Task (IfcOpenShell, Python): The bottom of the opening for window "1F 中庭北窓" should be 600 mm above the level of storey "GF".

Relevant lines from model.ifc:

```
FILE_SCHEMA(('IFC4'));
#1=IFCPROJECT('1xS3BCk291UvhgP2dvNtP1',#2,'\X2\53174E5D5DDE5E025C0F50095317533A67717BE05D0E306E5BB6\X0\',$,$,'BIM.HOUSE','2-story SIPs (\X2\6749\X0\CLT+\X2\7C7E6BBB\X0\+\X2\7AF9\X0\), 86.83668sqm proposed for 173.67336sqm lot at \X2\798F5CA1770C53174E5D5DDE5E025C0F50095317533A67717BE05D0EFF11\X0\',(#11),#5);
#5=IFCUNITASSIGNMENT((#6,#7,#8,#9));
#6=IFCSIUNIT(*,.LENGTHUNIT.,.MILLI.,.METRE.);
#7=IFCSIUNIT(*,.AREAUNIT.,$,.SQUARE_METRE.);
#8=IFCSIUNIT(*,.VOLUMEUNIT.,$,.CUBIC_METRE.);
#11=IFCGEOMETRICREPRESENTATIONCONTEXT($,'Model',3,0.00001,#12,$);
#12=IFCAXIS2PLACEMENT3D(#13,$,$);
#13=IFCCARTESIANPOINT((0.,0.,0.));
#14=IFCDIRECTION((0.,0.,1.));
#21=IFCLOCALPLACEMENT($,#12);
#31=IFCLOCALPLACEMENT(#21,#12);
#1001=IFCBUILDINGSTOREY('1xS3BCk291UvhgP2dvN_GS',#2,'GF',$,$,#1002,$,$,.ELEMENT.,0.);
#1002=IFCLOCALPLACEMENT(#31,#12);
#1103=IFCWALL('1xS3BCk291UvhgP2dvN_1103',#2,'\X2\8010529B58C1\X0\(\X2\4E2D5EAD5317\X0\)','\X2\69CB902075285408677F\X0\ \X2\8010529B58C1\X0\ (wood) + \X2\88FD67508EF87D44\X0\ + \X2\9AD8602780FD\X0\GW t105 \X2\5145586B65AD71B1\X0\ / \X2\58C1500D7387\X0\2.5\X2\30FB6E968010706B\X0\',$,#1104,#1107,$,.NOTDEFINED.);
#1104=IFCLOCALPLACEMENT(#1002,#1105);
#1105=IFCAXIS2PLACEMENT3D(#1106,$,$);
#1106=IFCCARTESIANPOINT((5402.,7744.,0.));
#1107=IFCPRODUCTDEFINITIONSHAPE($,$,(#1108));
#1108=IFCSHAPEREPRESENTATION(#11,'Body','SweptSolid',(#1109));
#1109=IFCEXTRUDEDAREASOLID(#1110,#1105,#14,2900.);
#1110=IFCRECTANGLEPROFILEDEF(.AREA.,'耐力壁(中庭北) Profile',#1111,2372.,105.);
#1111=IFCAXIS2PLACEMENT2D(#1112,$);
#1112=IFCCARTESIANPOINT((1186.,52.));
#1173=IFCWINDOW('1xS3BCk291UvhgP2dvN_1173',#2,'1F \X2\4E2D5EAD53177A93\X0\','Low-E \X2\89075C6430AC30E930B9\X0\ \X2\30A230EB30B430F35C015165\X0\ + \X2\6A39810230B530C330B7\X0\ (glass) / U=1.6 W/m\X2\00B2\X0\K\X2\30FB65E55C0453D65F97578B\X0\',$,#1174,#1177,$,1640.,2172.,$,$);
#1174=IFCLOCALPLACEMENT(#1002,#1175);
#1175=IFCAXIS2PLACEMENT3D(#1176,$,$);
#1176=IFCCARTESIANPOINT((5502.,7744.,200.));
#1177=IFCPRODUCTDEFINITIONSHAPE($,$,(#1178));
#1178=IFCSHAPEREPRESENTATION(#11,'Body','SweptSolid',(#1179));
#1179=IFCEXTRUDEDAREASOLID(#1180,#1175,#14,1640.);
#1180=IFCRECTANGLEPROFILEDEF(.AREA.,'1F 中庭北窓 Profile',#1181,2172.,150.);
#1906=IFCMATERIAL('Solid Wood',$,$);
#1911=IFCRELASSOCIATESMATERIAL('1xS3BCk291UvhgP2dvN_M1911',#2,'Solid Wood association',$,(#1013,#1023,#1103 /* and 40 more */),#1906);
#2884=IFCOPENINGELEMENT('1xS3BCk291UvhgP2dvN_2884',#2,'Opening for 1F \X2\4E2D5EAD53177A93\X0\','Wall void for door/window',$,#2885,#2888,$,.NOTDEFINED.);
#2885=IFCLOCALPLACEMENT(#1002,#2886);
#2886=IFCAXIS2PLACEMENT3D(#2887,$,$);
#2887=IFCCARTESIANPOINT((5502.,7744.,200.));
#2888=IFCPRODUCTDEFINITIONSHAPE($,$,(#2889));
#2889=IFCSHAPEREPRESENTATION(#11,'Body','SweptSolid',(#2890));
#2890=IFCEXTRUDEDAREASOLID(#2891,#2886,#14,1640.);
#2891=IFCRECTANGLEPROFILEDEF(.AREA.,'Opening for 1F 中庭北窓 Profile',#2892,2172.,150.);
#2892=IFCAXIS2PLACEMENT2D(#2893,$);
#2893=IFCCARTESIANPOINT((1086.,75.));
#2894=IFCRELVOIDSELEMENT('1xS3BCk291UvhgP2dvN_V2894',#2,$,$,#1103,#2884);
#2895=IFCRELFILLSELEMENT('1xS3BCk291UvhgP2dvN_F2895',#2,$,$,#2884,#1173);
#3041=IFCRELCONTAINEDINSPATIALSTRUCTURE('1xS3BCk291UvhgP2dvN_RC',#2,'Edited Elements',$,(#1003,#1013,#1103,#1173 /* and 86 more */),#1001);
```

```python
import numpy as np
import ifcopenshell
import ifcopenshell.api.geometry
import ifcopenshell.geom
import ifcopenshell.util.element
import ifcopenshell.util.placement
import ifcopenshell.util.shape
import ifcopenshell.util.unit

model = ifcopenshell.open("model.ifc")
unit_scale = ifcopenshell.util.unit.calculate_unit_scale(model)

window = model.by_guid("1xS3BCk291UvhgP2dvN_1173")
opening = window.FillsVoids[0].RelatingOpeningElement
storey = ifcopenshell.util.element.get_container(window, ifc_class="IfcBuildingStorey")
level = ifcopenshell.util.placement.get_local_placement(storey.ObjectPlacement)[2, 3]

# The opening's origin need not be at the sill, so measure its lowest point.
shape = ifcopenshell.geom.create_shape(ifcopenshell.geom.settings(), opening)
bottom = ifcopenshell.util.shape.get_shape_bottom_elevation(shape, shape.geometry) / unit_scale
dz = level + 0.6 / unit_scale - bottom

shift = np.array([0.0, 0.0, dz])
# The window is not placed relative to its opening, so move both.
for product in (opening, window):
    matrix = ifcopenshell.util.placement.get_local_placement(product.ObjectPlacement)
    matrix[:3, 3] += shift
    ifcopenshell.api.geometry.edit_object_placement(model, product=product, matrix=matrix, is_si=False)

print(f"moved by {dz * unit_scale:+.3f} m")

model.write("model_rev.ifc")
```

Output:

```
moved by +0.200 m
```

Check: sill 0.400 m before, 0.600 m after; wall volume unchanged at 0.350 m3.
